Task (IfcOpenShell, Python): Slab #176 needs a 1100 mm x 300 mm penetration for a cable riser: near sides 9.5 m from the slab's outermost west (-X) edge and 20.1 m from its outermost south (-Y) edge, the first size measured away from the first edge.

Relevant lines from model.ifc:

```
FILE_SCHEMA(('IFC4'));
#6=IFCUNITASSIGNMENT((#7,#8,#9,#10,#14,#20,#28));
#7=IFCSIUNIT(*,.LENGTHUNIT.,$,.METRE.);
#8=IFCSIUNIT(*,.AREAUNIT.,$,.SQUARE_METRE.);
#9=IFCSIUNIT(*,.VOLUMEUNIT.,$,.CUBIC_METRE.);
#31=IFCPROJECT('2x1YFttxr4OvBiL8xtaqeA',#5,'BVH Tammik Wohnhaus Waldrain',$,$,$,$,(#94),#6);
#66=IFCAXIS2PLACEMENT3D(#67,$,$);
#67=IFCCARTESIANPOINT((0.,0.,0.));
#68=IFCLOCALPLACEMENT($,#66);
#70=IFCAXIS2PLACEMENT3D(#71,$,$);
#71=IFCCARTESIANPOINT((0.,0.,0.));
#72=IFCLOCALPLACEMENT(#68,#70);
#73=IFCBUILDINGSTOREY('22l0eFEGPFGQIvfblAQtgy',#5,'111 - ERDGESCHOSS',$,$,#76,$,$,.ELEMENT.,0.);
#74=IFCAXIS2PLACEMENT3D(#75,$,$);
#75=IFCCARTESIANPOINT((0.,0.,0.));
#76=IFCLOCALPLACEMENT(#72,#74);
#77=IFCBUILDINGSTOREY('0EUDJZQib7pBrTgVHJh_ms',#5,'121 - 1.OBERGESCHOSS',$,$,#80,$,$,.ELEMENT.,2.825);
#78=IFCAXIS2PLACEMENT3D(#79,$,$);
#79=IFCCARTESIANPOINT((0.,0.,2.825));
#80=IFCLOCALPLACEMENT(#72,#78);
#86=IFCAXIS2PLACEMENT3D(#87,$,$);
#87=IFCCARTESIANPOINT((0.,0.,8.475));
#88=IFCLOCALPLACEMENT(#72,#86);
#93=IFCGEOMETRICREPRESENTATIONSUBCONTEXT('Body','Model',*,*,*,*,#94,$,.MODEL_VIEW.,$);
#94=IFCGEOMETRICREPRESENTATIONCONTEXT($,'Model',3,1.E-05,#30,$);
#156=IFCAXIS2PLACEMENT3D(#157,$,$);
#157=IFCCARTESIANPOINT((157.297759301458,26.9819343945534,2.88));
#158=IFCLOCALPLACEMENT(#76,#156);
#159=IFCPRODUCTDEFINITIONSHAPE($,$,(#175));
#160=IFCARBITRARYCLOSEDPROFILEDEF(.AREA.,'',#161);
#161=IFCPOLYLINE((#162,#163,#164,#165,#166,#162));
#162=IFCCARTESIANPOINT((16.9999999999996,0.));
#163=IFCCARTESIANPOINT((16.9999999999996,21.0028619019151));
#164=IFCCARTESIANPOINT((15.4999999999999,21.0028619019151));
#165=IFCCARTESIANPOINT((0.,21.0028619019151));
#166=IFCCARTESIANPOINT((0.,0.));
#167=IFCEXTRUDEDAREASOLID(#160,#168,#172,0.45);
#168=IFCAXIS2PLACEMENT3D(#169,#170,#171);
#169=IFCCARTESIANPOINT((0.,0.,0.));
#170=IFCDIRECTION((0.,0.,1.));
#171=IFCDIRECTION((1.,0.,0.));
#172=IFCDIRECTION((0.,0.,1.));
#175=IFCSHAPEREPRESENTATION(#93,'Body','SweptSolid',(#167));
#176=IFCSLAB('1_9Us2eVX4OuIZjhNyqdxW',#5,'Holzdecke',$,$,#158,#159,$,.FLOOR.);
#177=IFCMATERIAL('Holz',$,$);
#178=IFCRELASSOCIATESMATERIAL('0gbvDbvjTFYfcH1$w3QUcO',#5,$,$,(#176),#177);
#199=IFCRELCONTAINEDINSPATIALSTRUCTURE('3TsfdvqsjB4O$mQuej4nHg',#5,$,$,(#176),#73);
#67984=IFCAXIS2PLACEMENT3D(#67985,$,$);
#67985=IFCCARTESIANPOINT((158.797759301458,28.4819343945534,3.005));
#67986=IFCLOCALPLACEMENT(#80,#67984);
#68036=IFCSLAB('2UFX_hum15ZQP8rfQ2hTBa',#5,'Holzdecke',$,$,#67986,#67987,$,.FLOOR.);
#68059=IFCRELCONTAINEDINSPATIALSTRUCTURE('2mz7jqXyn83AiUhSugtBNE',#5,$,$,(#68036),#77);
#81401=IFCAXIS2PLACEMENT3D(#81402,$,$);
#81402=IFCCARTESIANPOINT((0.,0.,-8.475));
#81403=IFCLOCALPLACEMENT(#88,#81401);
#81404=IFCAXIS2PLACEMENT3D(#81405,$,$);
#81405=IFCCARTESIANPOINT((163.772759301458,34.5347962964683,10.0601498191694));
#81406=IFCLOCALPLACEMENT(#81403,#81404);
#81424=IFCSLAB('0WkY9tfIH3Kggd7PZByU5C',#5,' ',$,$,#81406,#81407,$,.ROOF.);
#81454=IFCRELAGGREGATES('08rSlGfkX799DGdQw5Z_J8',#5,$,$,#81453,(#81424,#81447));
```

```python
import numpy as np
import ifcopenshell
import ifcopenshell.api.feature
import ifcopenshell.api.geometry
import ifcopenshell.api.root
import ifcopenshell.geom
import ifcopenshell.util.placement
import ifcopenshell.util.representation
import ifcopenshell.util.shape
import ifcopenshell.util.unit

model = ifcopenshell.open("model.ifc")
unit_scale = ifcopenshell.util.unit.calculate_unit_scale(model)
settings = ifcopenshell.geom.settings()


def volume(element):
    """Net volume in cubic metres, openings subtracted."""
    shape = ifcopenshell.geom.create_shape(settings, element)
    return ifcopenshell.util.shape.get_volume(shape.geometry)


slab = model.by_guid("1_9Us2eVX4OuIZjhNyqdxW")
before = volume(slab)

# Extent in the slab's own axes, in metres. The edges named are its -X and -Y sides.
slab_shape = ifcopenshell.geom.create_shape(settings, slab)
vertices = ifcopenshell.util.shape.get_vertices(slab_shape.geometry)
x_min, y_min, bottom = vertices.min(axis=0)
top = vertices[:, 2].max()

opening = ifcopenshell.api.root.create_entity(model, ifc_class="IfcOpeningElement", name="Cable riser opening", predefined_type="OPENING")
context = ifcopenshell.util.representation.get_context(model, "Model", "Body", "MODEL_VIEW")
width, depth = 1.1, 0.3
outline = [(0.0, 0.0), (width, 0.0), (width, depth), (0.0, depth), (0.0, 0.0)]
# Overshoot both faces by 50 mm so the cut is clean.
shape = ifcopenshell.api.geometry.add_slab_representation(
    model, context=context, depth=top - bottom + 0.1, polyline=outline
)
ifcopenshell.api.geometry.assign_representation(model, product=opening, representation=shape)

matrix = ifcopenshell.util.placement.get_local_placement(slab.ObjectPlacement)
matrix[:, 3] = matrix @ np.append(np.array([x_min + 9.5, y_min + 20.1, bottom - 0.05]) / unit_scale, 1.0)
ifcopenshell.api.geometry.edit_object_placement(model, product=opening, matrix=matrix, is_si=False)
ifcopenshell.api.feature.add_feature(model, feature=opening, element=slab)

after = volume(slab)

print(f"slab volume {before:.3f} -> {after:.3f} m3")

model.write("model_updated.ifc")
```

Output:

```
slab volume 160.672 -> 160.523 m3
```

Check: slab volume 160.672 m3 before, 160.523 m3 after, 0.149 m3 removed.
